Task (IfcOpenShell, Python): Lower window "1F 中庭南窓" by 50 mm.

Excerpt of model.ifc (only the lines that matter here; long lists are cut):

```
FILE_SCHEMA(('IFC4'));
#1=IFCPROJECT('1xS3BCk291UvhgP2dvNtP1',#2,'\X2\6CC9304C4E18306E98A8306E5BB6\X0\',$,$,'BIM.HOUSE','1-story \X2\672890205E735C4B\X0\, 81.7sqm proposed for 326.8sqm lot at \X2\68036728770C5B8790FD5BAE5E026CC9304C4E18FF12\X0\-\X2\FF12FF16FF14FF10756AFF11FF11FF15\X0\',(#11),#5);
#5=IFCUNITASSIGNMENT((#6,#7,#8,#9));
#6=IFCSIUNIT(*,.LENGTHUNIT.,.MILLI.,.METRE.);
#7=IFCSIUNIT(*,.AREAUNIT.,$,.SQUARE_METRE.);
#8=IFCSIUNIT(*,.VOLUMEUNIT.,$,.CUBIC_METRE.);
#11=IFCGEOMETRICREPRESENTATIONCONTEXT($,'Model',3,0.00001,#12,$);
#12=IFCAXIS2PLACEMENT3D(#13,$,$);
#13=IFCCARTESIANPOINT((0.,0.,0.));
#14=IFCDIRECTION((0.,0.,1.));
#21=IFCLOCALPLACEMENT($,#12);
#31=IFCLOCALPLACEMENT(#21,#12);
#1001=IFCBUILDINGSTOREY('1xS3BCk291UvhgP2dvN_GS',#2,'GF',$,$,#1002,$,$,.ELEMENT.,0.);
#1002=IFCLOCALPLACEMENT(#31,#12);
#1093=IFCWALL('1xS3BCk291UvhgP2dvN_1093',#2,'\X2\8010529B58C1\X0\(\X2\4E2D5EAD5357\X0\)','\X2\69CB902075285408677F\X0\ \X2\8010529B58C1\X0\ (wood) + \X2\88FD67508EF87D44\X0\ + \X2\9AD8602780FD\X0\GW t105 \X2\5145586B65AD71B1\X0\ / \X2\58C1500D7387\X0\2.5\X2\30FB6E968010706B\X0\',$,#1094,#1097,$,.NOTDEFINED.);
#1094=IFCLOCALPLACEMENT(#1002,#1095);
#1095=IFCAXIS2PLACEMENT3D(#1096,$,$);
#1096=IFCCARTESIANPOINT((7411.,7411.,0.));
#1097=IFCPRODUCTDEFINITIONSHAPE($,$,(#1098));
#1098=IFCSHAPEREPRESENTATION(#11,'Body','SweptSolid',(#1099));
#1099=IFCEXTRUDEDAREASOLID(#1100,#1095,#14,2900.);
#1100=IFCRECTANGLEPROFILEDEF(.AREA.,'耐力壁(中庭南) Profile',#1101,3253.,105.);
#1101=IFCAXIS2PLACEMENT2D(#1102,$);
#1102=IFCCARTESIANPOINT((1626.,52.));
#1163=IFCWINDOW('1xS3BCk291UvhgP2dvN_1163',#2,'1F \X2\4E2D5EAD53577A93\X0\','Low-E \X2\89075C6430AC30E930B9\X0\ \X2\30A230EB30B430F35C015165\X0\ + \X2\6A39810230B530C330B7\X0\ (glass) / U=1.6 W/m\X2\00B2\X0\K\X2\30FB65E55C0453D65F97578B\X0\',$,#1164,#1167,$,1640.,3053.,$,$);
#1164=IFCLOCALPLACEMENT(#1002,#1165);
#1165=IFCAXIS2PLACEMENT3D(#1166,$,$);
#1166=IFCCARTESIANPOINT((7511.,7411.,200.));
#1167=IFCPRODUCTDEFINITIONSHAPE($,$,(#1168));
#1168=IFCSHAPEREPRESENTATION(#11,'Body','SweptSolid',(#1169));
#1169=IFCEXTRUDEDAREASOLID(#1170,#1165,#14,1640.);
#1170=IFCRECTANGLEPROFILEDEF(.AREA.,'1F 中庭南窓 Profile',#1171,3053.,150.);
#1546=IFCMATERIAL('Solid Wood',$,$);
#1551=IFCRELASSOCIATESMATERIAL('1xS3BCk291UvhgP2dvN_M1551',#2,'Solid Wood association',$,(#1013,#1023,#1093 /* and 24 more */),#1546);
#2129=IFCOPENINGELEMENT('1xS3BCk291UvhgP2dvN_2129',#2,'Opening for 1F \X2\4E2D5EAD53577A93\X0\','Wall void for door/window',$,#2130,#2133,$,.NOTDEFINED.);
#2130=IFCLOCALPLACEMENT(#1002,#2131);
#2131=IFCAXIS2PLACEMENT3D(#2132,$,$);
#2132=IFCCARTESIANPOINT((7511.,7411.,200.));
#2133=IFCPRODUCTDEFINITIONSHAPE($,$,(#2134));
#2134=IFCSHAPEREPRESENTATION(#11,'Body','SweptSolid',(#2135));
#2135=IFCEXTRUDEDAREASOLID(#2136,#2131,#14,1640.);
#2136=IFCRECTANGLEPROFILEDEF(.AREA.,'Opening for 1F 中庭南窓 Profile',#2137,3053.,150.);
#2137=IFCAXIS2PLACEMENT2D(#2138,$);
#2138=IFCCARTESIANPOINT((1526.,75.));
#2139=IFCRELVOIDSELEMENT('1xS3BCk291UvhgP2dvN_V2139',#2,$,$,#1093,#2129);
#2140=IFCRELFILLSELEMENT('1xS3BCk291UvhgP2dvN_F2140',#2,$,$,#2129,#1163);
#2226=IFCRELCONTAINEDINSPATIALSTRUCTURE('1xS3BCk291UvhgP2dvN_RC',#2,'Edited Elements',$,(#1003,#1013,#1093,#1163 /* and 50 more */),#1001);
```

```python
import numpy as np
import ifcopenshell
import ifcopenshell.api.geometry
import ifcopenshell.util.placement
import ifcopenshell.util.unit

model = ifcopenshell.open("model.ifc")
unit_scale = ifcopenshell.util.unit.calculate_unit_scale(model)

window = model.by_id(1163)
opening = window.FillsVoids[0].RelatingOpeningElement
dz = -0.05 / unit_scale

shift = np.array([0.0, 0.0, dz])
# The window is not placed relative to its opening, so move both.
for product in (opening, window):
    matrix = ifcopenshell.util.placement.get_local_placement(product.ObjectPlacement)
    matrix[:3, 3] += shift
    ifcopenshell.api.geometry.edit_object_placement(model, product=product, matrix=matrix, is_si=False)

print(f"moved by {dz * unit_scale:+.3f} m")

model.write("model_updated.ifc")
```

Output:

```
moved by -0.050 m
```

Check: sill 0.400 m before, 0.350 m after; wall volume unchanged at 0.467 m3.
